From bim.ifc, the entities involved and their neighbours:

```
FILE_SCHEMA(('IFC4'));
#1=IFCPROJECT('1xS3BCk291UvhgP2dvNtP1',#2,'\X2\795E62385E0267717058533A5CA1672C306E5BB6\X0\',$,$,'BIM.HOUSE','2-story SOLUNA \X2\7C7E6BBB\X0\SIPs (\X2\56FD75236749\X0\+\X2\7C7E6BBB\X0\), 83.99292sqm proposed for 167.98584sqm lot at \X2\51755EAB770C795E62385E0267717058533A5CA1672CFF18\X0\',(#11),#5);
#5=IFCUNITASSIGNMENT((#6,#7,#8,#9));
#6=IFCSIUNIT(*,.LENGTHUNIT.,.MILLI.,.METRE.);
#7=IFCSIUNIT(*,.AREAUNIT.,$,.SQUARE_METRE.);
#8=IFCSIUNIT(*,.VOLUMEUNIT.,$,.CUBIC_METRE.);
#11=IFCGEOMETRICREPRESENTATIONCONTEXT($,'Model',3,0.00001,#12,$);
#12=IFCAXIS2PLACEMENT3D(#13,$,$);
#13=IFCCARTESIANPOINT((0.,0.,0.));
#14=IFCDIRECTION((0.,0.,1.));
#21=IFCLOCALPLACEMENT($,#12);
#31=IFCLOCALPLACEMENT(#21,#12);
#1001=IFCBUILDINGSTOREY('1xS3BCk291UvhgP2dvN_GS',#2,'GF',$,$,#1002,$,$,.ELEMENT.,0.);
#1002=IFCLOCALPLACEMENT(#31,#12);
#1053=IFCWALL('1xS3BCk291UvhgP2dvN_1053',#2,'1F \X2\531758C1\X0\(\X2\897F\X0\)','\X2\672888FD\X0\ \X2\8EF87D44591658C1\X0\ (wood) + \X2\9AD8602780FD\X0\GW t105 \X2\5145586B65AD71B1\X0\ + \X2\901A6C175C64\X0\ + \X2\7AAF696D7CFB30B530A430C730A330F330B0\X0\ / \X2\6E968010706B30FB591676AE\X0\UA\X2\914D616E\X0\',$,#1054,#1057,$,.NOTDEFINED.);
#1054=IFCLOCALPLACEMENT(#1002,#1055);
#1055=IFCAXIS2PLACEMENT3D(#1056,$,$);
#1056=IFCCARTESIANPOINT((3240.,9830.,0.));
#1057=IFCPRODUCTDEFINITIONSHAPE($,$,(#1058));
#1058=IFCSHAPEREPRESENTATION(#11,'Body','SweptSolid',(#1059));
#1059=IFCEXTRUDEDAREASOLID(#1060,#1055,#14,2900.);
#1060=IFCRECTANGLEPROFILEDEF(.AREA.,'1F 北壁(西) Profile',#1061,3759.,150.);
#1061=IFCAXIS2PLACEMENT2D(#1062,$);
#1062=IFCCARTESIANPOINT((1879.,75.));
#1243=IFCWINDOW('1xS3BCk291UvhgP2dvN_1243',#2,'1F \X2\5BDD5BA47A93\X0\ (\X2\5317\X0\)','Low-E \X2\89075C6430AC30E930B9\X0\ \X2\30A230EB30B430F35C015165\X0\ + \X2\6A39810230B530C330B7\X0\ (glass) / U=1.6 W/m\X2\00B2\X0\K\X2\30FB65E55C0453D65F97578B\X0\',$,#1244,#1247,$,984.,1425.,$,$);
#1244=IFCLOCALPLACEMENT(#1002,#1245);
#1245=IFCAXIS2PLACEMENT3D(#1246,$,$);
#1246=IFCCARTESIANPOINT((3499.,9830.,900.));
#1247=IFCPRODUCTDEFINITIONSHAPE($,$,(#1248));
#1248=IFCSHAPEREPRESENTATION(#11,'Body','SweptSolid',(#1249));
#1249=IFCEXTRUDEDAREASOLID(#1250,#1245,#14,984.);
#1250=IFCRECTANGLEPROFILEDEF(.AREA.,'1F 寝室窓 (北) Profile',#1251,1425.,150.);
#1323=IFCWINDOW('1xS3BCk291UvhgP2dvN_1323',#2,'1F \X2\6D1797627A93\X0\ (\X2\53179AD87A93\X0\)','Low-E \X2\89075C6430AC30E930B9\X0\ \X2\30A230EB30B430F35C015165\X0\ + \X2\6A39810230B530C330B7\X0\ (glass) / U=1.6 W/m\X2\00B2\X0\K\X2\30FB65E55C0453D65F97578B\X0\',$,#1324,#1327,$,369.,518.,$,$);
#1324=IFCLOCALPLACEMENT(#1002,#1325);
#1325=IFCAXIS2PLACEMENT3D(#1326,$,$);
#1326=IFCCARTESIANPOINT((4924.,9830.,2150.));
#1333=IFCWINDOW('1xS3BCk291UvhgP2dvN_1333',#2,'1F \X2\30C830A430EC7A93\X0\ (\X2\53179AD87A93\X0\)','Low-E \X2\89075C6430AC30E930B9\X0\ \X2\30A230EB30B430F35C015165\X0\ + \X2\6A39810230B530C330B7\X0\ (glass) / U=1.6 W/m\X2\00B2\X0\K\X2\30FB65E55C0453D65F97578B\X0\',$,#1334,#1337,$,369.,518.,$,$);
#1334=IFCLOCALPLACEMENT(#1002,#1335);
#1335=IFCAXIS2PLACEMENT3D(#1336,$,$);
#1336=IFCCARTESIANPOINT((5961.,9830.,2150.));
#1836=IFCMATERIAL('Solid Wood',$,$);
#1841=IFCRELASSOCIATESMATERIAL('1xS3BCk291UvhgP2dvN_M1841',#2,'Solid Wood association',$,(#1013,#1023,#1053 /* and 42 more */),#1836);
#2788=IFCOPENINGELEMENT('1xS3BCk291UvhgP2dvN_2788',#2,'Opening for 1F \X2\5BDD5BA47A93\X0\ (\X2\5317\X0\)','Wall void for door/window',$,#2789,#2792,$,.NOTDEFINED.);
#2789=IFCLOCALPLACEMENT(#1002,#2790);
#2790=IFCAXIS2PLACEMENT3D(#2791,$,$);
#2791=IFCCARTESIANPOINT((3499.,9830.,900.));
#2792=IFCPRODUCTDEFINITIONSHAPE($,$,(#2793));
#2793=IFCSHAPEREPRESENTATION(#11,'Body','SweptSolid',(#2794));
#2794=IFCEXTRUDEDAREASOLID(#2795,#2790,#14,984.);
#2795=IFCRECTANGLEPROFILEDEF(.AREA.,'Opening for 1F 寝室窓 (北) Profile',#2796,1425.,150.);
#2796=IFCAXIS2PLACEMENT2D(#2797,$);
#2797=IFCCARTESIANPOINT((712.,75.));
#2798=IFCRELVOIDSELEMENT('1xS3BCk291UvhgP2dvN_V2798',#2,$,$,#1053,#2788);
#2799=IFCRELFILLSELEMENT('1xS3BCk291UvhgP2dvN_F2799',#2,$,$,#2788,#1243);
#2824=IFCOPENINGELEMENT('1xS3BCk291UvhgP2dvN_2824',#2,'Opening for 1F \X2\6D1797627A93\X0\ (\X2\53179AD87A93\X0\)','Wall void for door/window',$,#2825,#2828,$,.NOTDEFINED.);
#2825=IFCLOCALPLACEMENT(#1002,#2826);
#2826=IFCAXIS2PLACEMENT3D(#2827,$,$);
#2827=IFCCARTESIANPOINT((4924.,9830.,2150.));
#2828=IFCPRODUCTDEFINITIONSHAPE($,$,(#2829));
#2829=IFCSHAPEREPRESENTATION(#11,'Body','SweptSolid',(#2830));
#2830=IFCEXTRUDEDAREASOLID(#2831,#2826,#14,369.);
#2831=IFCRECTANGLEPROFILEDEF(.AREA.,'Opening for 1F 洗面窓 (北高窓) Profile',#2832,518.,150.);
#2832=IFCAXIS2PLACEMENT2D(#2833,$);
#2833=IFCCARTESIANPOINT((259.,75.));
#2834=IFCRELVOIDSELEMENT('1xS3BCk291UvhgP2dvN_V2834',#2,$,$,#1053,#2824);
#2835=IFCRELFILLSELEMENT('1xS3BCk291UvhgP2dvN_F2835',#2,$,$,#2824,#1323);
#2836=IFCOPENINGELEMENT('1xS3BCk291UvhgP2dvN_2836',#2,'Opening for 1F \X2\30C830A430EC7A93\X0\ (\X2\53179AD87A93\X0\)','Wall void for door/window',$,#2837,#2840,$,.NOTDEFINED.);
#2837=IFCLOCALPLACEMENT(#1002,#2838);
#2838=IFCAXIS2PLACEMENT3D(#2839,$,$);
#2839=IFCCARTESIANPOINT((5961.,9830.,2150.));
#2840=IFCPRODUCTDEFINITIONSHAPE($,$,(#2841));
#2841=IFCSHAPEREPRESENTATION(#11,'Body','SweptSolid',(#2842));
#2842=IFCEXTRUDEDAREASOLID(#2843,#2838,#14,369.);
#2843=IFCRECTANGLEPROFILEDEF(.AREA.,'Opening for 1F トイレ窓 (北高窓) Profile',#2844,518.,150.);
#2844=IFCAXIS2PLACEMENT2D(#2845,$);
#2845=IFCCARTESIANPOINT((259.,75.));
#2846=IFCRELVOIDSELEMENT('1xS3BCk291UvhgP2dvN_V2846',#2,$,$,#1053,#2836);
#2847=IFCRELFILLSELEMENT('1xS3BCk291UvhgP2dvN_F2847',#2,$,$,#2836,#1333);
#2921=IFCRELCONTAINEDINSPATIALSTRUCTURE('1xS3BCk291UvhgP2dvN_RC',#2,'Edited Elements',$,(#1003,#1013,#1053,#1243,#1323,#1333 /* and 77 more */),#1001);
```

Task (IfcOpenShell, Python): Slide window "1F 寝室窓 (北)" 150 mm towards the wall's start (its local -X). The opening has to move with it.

```python
import ifcopenshell
import ifcopenshell.api.geometry
import ifcopenshell.util.placement
import ifcopenshell.util.unit

model = ifcopenshell.open("bim.ifc")
unit_scale = ifcopenshell.util.unit.calculate_unit_scale(model)

window = model.by_guid("1xS3BCk291UvhgP2dvN_1243")
opening = window.FillsVoids[0].RelatingOpeningElement
wall = opening.VoidsElements[0].RelatingBuildingElement

wall_matrix = ifcopenshell.util.placement.get_local_placement(wall.ObjectPlacement)
shift = wall_matrix[:3, 0] * -0.15 / unit_scale
before = ifcopenshell.util.placement.get_local_placement(window.ObjectPlacement)[:3, 3].copy()

# The window is not placed relative to its opening, so move both.
for product in (opening, window):
    matrix = ifcopenshell.util.placement.get_local_placement(product.ObjectPlacement)
    matrix[:3, 3] += shift
    ifcopenshell.api.geometry.edit_object_placement(model, product=product, matrix=matrix, is_si=False)

after = ifcopenshell.util.placement.get_local_placement(window.ObjectPlacement)[:3, 3]
print("window moved by", (after - before).round(3) + 0.0)

model.write("bim_v2.ifc")
```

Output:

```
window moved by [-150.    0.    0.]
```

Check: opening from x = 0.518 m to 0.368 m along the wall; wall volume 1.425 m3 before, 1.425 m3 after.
